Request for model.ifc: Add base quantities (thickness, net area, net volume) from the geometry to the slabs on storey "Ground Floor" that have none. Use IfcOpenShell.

First a look at what the model holds.

```python
import ifcopenshell
import ifcopenshell.util.element
import ifcopenshell.util.unit

model = ifcopenshell.open("model.ifc")
print(model.schema)
for unit_type in ("LENGTHUNIT", "AREAUNIT", "VOLUMEUNIT"):
    print(unit_type, ifcopenshell.util.unit.calculate_unit_scale(model, unit_type))
storey = next(s for s in model.by_type("IfcBuildingStorey") if s.Name == "Ground Floor")
slabs = [e for e in ifcopenshell.util.element.get_decomposition(storey) if e.is_a("IfcSlab")]
for e in sorted(slabs, key=lambda e: e.id()):
    print(e.id(), e.is_a(), e.Name, list(ifcopenshell.util.element.get_psets(e, qtos_only=True)), sep=" | ")
```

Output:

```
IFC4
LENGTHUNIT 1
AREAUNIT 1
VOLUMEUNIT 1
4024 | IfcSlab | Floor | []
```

```python
import ifcopenshell
import ifcopenshell.api.pset
import ifcopenshell.geom
import ifcopenshell.util.element
import ifcopenshell.util.shape
import ifcopenshell.util.unit

model = ifcopenshell.open("model.ifc")
unit_scale = ifcopenshell.util.unit.calculate_unit_scale(model)
area_scale = ifcopenshell.util.unit.calculate_unit_scale(model, "AREAUNIT")
volume_scale = ifcopenshell.util.unit.calculate_unit_scale(model, "VOLUMEUNIT")
settings = ifcopenshell.geom.settings()

storey = next(s for s in model.by_type("IfcBuildingStorey") if s.Name == "Ground Floor")
slabs = [e for e in ifcopenshell.util.element.get_decomposition(storey) if e.is_a("IfcSlab")]

for e in sorted(slabs, key=lambda e: e.id()):
    if ifcopenshell.util.element.get_psets(e, qtos_only=True, should_inherit=False):
        continue
    # Geometry comes back in metres, in the element's own axes.
    shape = ifcopenshell.geom.create_shape(settings, e)
    values = {
        "Width": ifcopenshell.util.shape.get_z(shape.geometry) / unit_scale,
        "NetArea": ifcopenshell.util.shape.get_footprint_area(shape.geometry) / area_scale,
        "NetVolume": ifcopenshell.util.shape.get_volume(shape.geometry) / volume_scale,
    }
    qto = ifcopenshell.api.pset.add_qto(model, product=e, name="Qto_SlabBaseQuantities")
    ifcopenshell.api.pset.edit_qto(model, qto=qto, properties=values)
    print(e.id(), {k: round(v, 3) for k, v in values.items()})

model.write("model_v2.ifc")
```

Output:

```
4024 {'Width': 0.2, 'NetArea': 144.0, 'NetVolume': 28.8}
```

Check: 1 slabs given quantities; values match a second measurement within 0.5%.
